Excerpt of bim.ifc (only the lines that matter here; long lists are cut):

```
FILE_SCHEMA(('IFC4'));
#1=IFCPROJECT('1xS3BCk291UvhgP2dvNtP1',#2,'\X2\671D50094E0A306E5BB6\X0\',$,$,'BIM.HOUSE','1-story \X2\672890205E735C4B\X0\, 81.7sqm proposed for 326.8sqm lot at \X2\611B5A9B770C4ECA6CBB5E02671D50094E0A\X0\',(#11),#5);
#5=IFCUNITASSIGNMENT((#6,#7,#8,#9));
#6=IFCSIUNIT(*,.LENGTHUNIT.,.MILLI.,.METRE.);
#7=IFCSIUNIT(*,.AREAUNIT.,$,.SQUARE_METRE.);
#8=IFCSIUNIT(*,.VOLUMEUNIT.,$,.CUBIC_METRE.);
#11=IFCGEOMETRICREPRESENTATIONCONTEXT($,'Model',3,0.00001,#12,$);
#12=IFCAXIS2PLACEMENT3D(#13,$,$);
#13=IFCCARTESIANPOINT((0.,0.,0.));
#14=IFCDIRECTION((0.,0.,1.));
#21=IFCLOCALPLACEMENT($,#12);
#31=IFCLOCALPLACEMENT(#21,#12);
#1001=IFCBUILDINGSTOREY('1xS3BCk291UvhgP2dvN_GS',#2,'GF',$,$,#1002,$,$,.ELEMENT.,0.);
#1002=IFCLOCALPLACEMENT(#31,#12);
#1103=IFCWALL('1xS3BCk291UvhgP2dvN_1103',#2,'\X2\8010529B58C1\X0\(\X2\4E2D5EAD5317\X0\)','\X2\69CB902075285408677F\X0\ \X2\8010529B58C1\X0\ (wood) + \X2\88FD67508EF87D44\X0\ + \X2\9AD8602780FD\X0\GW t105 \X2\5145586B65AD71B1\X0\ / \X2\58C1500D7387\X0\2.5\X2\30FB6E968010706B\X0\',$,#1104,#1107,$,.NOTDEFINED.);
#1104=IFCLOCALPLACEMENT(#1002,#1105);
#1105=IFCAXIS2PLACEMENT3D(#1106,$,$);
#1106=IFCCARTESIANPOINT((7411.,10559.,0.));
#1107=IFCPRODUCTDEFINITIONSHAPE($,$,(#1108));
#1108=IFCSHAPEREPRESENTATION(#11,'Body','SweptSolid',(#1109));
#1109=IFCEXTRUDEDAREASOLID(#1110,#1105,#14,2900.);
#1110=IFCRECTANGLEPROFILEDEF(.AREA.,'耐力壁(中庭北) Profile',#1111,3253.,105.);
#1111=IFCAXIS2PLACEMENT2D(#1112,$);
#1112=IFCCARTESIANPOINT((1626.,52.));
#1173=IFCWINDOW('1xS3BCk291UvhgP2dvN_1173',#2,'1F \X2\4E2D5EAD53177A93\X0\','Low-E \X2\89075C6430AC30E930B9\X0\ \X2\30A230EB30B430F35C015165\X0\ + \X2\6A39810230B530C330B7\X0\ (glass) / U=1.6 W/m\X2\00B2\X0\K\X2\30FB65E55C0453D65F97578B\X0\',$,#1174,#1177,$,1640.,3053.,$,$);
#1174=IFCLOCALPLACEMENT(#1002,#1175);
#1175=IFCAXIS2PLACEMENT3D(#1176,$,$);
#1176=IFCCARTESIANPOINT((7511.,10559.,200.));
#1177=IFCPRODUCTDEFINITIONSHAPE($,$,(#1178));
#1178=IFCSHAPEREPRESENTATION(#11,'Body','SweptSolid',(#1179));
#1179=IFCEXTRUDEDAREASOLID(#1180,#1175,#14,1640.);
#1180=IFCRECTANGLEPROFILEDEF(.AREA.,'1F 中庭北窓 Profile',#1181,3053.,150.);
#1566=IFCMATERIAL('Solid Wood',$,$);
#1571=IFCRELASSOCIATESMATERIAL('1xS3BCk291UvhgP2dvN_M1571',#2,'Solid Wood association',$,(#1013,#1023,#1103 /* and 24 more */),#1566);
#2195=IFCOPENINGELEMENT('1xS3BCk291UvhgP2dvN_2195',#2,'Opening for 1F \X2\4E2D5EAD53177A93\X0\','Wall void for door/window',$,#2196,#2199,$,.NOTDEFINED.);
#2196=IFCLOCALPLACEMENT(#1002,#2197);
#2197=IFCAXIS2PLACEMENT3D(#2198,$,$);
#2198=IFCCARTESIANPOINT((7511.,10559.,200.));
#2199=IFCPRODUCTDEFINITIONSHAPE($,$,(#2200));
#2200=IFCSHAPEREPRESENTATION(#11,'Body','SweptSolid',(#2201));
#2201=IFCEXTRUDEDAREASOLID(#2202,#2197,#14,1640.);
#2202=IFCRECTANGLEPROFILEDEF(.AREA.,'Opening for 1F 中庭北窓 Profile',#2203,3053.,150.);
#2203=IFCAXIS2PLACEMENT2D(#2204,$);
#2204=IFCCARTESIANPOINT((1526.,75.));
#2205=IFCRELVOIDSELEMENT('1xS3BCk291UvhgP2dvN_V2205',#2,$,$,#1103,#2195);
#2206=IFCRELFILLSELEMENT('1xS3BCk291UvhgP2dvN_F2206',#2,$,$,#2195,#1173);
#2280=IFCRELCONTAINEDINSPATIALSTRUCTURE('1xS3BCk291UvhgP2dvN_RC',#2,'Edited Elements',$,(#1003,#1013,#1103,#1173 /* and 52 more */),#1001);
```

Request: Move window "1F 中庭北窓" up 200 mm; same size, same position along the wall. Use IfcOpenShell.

```python
import numpy as np
import ifcopenshell
import ifcopenshell.api.geometry
import ifcopenshell.util.placement
import ifcopenshell.util.unit

model = ifcopenshell.open("bim.ifc")
unit_scale = ifcopenshell.util.unit.calculate_unit_scale(model)

window = model.by_guid("1xS3BCk291UvhgP2dvN_1173")
opening = window.FillsVoids[0].RelatingOpeningElement
dz = 0.2 / unit_scale

shift = np.array([0.0, 0.0, dz])
# The window is not placed relative to its opening, so move both.
for product in (opening, window):
    matrix = ifcopenshell.util.placement.get_local_placement(product.ObjectPlacement)
    matrix[:3, 3] += shift
    ifcopenshell.api.geometry.edit_object_placement(model, product=product, matrix=matrix, is_si=False)

print(f"moved by {dz * unit_scale:+.3f} m")

model.write("bim_updated.ifc")
```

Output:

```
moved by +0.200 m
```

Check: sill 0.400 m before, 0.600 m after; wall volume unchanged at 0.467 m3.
